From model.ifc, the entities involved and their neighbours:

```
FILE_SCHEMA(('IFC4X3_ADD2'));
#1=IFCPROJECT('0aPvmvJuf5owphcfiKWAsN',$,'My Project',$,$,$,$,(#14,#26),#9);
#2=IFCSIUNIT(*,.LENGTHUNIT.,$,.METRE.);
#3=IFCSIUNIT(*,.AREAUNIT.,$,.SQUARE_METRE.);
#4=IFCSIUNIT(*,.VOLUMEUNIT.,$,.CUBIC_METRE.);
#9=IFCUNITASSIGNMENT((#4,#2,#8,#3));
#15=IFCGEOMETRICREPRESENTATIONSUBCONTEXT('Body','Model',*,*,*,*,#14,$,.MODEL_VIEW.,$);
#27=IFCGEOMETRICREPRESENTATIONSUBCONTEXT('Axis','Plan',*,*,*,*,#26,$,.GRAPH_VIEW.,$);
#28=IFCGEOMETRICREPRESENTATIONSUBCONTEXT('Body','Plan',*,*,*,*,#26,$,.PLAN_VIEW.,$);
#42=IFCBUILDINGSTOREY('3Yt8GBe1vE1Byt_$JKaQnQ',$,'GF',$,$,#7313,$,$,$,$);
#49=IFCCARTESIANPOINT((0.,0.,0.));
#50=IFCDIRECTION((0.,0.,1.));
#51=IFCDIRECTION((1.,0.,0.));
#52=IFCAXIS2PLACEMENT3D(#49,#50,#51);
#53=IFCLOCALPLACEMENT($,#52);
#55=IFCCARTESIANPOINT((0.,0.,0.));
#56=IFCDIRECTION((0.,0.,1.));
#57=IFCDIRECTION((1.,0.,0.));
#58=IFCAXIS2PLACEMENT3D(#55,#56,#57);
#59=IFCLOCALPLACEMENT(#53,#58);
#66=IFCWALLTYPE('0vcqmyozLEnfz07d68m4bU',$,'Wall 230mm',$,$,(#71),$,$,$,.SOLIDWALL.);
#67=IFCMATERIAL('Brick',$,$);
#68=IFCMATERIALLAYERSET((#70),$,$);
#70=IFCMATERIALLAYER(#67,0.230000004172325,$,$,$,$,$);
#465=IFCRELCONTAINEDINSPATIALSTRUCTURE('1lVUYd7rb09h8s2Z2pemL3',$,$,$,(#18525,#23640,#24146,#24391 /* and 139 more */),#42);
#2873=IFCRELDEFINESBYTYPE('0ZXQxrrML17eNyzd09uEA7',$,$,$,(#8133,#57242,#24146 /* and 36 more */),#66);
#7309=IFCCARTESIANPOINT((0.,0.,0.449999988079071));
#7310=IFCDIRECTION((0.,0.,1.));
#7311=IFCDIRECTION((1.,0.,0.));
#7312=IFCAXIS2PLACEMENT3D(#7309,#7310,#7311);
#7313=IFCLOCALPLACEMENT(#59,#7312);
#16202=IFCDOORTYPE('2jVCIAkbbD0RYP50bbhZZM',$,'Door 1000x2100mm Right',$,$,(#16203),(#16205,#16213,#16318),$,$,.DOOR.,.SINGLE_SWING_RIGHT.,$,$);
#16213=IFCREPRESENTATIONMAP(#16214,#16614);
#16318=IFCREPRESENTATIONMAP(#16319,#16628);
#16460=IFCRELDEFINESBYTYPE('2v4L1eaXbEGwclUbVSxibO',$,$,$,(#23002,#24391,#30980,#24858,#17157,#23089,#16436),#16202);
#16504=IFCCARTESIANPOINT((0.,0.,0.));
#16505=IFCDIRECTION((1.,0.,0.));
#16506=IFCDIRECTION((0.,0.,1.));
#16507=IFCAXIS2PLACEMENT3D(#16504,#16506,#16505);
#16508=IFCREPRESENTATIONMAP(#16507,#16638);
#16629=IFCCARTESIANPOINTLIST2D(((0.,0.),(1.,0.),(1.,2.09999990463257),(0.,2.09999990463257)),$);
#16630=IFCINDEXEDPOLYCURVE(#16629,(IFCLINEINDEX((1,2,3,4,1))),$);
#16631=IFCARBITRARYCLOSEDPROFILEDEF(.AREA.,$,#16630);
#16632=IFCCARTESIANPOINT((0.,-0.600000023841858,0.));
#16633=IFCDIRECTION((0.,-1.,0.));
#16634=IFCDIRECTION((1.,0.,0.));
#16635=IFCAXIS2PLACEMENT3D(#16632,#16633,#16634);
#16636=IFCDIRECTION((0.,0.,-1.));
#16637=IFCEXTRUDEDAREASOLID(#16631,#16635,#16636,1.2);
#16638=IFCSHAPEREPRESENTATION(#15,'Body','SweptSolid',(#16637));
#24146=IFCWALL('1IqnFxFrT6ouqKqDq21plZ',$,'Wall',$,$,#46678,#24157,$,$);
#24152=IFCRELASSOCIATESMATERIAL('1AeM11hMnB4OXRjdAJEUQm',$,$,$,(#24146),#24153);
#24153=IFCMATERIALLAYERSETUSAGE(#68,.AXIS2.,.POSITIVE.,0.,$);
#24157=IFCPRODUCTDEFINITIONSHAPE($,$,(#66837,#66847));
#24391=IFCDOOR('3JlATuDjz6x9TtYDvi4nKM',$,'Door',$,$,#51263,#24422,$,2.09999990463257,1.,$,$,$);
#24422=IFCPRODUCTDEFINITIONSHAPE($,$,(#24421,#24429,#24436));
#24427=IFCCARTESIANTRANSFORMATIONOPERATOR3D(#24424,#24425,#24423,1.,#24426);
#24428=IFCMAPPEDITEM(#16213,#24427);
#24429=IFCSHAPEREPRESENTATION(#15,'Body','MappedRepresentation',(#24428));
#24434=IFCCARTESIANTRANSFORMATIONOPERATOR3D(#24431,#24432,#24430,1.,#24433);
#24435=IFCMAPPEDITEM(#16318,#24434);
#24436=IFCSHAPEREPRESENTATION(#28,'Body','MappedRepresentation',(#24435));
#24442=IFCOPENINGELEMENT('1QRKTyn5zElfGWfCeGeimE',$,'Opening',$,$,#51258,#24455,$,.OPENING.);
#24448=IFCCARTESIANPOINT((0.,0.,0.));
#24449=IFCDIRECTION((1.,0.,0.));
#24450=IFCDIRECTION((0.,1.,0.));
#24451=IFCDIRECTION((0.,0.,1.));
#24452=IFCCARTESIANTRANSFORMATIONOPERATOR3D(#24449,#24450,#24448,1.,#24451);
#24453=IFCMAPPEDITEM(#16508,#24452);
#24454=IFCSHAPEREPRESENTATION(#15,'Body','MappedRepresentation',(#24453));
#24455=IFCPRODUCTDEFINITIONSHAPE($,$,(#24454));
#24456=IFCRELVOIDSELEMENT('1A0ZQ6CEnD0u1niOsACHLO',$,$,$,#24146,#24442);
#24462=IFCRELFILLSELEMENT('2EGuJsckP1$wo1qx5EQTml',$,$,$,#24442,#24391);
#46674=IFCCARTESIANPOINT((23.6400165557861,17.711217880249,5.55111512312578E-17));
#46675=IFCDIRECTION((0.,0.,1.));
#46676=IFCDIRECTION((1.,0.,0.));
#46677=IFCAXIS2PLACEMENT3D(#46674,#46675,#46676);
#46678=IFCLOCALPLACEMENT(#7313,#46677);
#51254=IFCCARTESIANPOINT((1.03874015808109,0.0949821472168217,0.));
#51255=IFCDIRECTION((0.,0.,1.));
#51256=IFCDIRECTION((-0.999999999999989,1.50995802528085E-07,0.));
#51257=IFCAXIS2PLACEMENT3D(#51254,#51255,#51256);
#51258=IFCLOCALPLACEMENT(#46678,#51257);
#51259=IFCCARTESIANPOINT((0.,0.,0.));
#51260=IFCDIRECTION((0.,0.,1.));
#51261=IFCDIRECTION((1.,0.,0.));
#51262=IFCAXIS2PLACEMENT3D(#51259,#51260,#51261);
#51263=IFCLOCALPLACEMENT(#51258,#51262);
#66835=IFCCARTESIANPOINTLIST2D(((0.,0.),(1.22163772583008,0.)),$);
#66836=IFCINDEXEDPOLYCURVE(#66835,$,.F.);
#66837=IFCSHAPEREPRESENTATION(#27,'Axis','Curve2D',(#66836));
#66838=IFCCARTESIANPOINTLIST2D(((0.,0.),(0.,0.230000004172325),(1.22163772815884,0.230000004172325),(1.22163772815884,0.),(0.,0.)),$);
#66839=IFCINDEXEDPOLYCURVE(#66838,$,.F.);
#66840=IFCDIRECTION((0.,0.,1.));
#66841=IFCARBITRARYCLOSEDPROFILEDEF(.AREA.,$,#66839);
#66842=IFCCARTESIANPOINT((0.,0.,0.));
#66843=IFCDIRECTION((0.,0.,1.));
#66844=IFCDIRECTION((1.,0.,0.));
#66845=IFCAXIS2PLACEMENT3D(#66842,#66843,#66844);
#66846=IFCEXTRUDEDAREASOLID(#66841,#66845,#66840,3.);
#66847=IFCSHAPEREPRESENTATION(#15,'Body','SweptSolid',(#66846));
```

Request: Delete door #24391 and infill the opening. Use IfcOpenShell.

```python
import ifcopenshell
import ifcopenshell.api.feature
import ifcopenshell.api.root
import ifcopenshell.geom
import ifcopenshell.util.shape

model = ifcopenshell.open("model.ifc")
settings = ifcopenshell.geom.settings()


def volume(element):
    """Net volume in cubic metres, openings subtracted."""
    shape = ifcopenshell.geom.create_shape(settings, element)
    return ifcopenshell.util.shape.get_volume(shape.geometry)


door = model.by_guid("3JlATuDjz6x9TtYDvi4nKM")
opening = door.FillsVoids[0].RelatingOpeningElement
wall = opening.VoidsElements[0].RelatingBuildingElement
before = volume(wall)

ifcopenshell.api.root.remove_product(model, product=door)
ifcopenshell.api.feature.remove_feature(model, feature=opening)

after = volume(wall)

print(f"wall volume {before:.3f} -> {after:.3f} m3")

model.write("model_v2.ifc")
```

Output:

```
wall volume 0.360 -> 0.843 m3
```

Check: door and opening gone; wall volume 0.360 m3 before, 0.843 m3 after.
